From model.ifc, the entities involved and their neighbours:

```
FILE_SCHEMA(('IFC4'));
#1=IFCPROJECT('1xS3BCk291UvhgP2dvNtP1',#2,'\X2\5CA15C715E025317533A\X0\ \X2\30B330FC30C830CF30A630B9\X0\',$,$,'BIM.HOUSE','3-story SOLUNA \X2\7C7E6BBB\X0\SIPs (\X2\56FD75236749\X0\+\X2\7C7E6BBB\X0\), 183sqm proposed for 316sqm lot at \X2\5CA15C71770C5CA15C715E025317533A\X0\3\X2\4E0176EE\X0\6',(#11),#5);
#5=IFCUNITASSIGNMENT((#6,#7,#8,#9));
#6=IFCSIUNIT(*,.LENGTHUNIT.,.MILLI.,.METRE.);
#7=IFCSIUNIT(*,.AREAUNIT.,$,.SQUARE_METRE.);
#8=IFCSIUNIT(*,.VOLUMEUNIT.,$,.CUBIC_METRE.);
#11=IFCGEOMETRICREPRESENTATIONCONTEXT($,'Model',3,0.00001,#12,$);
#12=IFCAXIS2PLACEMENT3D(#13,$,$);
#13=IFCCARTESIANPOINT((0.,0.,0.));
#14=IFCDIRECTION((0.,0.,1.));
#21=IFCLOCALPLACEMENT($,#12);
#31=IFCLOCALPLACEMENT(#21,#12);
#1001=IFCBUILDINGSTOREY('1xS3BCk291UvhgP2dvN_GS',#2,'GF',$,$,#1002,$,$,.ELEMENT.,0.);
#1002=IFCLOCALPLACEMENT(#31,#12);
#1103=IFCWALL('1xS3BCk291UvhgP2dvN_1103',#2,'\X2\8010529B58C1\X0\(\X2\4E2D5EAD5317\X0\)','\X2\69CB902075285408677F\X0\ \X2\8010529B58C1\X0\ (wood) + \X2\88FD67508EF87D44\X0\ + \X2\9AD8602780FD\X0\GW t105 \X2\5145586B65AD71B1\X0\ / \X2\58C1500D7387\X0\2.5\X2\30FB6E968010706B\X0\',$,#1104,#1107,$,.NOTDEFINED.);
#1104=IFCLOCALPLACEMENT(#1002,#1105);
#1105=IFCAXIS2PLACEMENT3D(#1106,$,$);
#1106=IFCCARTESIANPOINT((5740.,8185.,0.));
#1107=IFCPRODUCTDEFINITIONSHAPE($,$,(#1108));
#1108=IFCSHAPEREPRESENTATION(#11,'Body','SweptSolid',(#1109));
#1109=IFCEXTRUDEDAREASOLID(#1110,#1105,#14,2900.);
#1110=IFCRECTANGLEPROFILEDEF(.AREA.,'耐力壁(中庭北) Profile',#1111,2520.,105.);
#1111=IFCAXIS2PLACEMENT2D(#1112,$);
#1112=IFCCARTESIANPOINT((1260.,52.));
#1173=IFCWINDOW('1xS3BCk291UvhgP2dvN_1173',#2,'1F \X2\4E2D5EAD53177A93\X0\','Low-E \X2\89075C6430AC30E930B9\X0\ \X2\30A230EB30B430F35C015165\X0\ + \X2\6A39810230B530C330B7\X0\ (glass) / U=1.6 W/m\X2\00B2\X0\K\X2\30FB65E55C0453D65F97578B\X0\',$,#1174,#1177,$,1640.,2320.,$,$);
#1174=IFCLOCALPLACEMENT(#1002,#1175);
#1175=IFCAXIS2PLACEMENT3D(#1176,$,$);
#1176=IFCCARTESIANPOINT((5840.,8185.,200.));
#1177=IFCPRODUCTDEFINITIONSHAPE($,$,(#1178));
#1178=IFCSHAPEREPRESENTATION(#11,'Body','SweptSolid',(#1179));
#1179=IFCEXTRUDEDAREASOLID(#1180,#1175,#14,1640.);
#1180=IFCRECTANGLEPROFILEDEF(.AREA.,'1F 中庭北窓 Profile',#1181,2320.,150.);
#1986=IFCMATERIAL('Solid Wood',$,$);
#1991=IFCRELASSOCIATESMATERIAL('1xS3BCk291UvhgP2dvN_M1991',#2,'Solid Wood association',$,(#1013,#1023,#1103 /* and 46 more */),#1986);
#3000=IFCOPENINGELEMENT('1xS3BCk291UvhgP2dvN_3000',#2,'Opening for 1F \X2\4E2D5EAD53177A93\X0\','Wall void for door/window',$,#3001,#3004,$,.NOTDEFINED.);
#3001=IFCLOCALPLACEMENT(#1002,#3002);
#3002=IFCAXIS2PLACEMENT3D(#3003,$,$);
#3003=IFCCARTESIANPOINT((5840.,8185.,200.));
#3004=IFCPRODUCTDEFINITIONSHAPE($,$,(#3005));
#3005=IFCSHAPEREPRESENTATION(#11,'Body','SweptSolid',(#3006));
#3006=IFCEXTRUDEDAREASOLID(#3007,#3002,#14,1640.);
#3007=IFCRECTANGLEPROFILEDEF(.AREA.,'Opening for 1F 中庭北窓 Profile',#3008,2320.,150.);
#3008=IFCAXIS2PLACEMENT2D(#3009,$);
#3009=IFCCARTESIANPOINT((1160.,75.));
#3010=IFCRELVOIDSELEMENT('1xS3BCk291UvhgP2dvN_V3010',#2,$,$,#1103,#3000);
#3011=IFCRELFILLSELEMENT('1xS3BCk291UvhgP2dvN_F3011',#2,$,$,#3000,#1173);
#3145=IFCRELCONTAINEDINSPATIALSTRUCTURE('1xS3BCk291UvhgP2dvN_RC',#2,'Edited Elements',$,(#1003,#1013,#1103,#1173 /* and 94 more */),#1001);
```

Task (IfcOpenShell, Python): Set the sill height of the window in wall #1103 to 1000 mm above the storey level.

```python
import numpy as np
import ifcopenshell
import ifcopenshell.api.geometry
import ifcopenshell.geom
import ifcopenshell.util.element
import ifcopenshell.util.placement
import ifcopenshell.util.shape
import ifcopenshell.util.unit

model = ifcopenshell.open("model.ifc")
unit_scale = ifcopenshell.util.unit.calculate_unit_scale(model)

window = model.by_guid("1xS3BCk291UvhgP2dvN_1173")
opening = window.FillsVoids[0].RelatingOpeningElement
storey = ifcopenshell.util.element.get_container(window, ifc_class="IfcBuildingStorey")
level = ifcopenshell.util.placement.get_local_placement(storey.ObjectPlacement)[2, 3]

# The opening's origin need not be at the sill, so measure its lowest point.
shape = ifcopenshell.geom.create_shape(ifcopenshell.geom.settings(), opening)
bottom = ifcopenshell.util.shape.get_shape_bottom_elevation(shape, shape.geometry) / unit_scale
dz = level + 1000.0 - bottom

shift = np.array([0.0, 0.0, dz])
# The window is not placed relative to its opening, so move both.
for product in (opening, window):
    matrix = ifcopenshell.util.placement.get_local_placement(product.ObjectPlacement)
    matrix[:3, 3] += shift
    ifcopenshell.api.geometry.edit_object_placement(model, product=product, matrix=matrix, is_si=False)

print(f"moved by {dz * unit_scale:+.3f} m")

model.write("model-out.ifc")
```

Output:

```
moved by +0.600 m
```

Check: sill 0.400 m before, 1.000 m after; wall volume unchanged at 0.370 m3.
